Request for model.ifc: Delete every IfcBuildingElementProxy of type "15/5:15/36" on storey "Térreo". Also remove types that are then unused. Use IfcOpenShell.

First a look at what the model holds.

```python
import ifcopenshell
import ifcopenshell.util.element

model = ifcopenshell.open("model.ifc")
print(model.schema)
storey = next(s for s in model.by_type("IfcBuildingStorey") if s.Name == "Térreo")
proxies = [e for e in ifcopenshell.util.element.get_decomposition(storey) if e.is_a("IfcBuildingElementProxy")]
seen = {}
for e in proxies:
    element_type = ifcopenshell.util.element.get_type(e)
    name = element_type.Name if element_type not in (None, e) else None
    seen[name] = seen.get(name, 0) + 1
for name, count in sorted(seen.items(), key=str):
    print(count, "x", name)
```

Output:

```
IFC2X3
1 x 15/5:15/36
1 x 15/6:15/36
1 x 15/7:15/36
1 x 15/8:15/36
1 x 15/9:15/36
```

```python
import ifcopenshell
import ifcopenshell.api.root
import ifcopenshell.util.element

model = ifcopenshell.open("model.ifc")

storey = next(s for s in model.by_type("IfcBuildingStorey") if s.Name == "Térreo")
proxies = [e for e in ifcopenshell.util.element.get_decomposition(storey) if e.is_a("IfcBuildingElementProxy")]
targets = [e for e in proxies if (t := ifcopenshell.util.element.get_type(e)) not in (None, e) and t.Name == "15/5:15/36"]
types = {ifcopenshell.util.element.get_type(e) for e in targets} - {None, *targets}

for e in targets:
    ifcopenshell.api.root.remove_product(model, product=e)
print(len(targets), "removed")

unused = [t for t in types if not ifcopenshell.util.element.get_types(t)]
for t in unused:
    ifcopenshell.api.root.remove_product(model, product=t)
print(len(unused), "unused types removed")

model.write("model_edited.ifc")
```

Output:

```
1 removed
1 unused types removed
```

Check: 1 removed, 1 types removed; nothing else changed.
